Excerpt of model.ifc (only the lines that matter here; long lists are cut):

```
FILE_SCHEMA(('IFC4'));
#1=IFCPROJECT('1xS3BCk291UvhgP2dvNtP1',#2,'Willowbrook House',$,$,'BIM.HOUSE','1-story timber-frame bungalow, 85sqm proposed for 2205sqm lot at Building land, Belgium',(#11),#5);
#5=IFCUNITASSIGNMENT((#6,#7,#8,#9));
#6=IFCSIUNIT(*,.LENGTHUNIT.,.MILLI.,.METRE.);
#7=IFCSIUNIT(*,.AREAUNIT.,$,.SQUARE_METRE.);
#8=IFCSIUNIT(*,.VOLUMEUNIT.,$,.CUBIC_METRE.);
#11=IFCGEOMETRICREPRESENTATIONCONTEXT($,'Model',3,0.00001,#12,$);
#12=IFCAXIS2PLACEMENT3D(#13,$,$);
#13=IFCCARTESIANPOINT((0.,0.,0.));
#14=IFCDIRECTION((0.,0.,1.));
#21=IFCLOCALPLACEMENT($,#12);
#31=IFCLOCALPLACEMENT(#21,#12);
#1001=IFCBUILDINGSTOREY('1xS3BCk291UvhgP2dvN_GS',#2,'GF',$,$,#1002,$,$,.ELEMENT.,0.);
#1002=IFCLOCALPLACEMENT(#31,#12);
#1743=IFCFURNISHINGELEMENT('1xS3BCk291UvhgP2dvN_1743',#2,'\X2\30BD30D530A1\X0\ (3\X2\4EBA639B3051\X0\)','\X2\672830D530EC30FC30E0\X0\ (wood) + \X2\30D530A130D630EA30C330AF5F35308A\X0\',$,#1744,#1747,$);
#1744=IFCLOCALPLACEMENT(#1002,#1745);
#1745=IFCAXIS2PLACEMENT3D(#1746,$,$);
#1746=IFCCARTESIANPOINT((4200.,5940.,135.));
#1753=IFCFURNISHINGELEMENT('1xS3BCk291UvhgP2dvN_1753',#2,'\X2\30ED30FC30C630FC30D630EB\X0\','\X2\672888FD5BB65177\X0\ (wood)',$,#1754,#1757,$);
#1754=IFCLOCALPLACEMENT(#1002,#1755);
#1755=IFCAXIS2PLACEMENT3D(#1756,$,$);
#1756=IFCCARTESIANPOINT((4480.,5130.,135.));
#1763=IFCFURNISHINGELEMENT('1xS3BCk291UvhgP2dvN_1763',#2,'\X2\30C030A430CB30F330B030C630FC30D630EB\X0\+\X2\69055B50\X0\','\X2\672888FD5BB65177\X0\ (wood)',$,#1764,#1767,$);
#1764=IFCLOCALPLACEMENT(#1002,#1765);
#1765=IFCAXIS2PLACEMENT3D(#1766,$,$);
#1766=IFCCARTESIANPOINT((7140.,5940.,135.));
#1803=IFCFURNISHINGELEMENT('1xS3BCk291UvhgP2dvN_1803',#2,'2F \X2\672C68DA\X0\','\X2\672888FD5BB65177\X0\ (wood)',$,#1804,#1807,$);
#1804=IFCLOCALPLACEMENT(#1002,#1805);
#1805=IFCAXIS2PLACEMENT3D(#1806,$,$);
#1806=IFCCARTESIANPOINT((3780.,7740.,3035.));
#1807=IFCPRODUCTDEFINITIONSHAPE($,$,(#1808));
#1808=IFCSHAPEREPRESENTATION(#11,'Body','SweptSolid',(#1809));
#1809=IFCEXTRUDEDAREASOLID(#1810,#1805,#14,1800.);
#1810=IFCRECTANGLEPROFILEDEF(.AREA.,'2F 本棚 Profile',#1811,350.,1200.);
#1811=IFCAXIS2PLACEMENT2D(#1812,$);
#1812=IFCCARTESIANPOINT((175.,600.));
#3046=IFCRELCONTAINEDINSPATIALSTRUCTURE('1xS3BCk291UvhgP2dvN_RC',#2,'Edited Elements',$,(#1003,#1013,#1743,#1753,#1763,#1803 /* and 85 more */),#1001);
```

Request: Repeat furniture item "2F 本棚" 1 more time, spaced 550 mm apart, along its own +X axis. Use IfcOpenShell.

```python
import ifcopenshell
import ifcopenshell.api.geometry
import ifcopenshell.api.root
import ifcopenshell.util.element
import ifcopenshell.util.placement

model = ifcopenshell.open("model.ifc")


def reuse_history(source, copy):
    """copy_class also copies each property set's owner history, people and application; keep the originals."""
    for rel in copy.IsDefinedBy:
        if rel.is_a("IfcRelDefinesByProperties") and (history := rel.RelatingPropertyDefinition.OwnerHistory):
            rel.RelatingPropertyDefinition.OwnerHistory = source.OwnerHistory
            ifcopenshell.util.element.remove_deep2(model, history)


source = model.by_id(1803)
base = ifcopenshell.util.placement.get_local_placement(source.ObjectPlacement)
step = base[:3, 0] * 550.0

for i in range(1, 2):
    copy = ifcopenshell.api.root.copy_class(model, product=source)
    copy.Representation = ifcopenshell.util.element.copy_deep(
        model, source.Representation, exclude=["IfcGeometricRepresentationContext", "IfcRepresentationMap"]
    )
    reuse_history(source, copy)
    matrix = base.copy()
    matrix[:3, 3] += i * step
    print("added at", matrix[:3, 3].round(3) + 0.0)
    ifcopenshell.api.geometry.edit_object_placement(model, product=copy, matrix=matrix, is_si=False)

model.write("model_v2.ifc")
```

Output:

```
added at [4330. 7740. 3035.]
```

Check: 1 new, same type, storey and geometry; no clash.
